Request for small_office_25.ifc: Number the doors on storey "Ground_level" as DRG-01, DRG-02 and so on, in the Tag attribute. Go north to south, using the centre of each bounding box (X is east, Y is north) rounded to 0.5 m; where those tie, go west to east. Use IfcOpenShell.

First a look at what the model holds.

```python
import ifcopenshell
import ifcopenshell.util.element
import ifcopenshell.util.placement

model = ifcopenshell.open("small_office_25.ifc")
print(model.schema)
storey = next(s for s in model.by_type("IfcBuildingStorey") if s.Name == "Ground_level")
doors = [e for e in ifcopenshell.util.element.get_decomposition(storey) if e.is_a("IfcDoor")]
for e in sorted(doors, key=lambda e: e.id()):
    origin = ifcopenshell.util.placement.get_local_placement(e.ObjectPlacement)[:3, 3]
    print(e.id(), e.Tag, e.Name, origin.round(2) + 0.0, sep=" | ")
```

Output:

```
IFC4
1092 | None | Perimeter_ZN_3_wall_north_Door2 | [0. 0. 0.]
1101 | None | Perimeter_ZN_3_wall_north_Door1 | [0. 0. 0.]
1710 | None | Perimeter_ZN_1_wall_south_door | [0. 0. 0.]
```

```python
import ifcopenshell
import ifcopenshell.geom
import ifcopenshell.util.element
import ifcopenshell.util.shape

model = ifcopenshell.open("small_office_25.ifc")
settings = ifcopenshell.geom.settings()
settings.set("use-world-coords", True)


def centre(element):
    shape = ifcopenshell.geom.create_shape(settings, element)
    return ifcopenshell.util.shape.get_bbox_centroid(shape.geometry)


storey = next(s for s in model.by_type("IfcBuildingStorey") if s.Name == "Ground_level")
doors = [e for e in ifcopenshell.util.element.get_decomposition(storey) if e.is_a("IfcDoor")]

# Insertion points can sit at a corner or the storey origin, so sort by the geometry (in metres).
centres = {e: centre(e) for e in doors}
doors.sort(key=lambda e: (-round(centres[e][1] / 0.5), centres[e][0]))

for i, e in enumerate(doors, start=1):
    number = f"DRG-{i:02d}"
    e.Tag = number
    print(e.id(), number)

model.write("small_office_25_edited.ifc")
```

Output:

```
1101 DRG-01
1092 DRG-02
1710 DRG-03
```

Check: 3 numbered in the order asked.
